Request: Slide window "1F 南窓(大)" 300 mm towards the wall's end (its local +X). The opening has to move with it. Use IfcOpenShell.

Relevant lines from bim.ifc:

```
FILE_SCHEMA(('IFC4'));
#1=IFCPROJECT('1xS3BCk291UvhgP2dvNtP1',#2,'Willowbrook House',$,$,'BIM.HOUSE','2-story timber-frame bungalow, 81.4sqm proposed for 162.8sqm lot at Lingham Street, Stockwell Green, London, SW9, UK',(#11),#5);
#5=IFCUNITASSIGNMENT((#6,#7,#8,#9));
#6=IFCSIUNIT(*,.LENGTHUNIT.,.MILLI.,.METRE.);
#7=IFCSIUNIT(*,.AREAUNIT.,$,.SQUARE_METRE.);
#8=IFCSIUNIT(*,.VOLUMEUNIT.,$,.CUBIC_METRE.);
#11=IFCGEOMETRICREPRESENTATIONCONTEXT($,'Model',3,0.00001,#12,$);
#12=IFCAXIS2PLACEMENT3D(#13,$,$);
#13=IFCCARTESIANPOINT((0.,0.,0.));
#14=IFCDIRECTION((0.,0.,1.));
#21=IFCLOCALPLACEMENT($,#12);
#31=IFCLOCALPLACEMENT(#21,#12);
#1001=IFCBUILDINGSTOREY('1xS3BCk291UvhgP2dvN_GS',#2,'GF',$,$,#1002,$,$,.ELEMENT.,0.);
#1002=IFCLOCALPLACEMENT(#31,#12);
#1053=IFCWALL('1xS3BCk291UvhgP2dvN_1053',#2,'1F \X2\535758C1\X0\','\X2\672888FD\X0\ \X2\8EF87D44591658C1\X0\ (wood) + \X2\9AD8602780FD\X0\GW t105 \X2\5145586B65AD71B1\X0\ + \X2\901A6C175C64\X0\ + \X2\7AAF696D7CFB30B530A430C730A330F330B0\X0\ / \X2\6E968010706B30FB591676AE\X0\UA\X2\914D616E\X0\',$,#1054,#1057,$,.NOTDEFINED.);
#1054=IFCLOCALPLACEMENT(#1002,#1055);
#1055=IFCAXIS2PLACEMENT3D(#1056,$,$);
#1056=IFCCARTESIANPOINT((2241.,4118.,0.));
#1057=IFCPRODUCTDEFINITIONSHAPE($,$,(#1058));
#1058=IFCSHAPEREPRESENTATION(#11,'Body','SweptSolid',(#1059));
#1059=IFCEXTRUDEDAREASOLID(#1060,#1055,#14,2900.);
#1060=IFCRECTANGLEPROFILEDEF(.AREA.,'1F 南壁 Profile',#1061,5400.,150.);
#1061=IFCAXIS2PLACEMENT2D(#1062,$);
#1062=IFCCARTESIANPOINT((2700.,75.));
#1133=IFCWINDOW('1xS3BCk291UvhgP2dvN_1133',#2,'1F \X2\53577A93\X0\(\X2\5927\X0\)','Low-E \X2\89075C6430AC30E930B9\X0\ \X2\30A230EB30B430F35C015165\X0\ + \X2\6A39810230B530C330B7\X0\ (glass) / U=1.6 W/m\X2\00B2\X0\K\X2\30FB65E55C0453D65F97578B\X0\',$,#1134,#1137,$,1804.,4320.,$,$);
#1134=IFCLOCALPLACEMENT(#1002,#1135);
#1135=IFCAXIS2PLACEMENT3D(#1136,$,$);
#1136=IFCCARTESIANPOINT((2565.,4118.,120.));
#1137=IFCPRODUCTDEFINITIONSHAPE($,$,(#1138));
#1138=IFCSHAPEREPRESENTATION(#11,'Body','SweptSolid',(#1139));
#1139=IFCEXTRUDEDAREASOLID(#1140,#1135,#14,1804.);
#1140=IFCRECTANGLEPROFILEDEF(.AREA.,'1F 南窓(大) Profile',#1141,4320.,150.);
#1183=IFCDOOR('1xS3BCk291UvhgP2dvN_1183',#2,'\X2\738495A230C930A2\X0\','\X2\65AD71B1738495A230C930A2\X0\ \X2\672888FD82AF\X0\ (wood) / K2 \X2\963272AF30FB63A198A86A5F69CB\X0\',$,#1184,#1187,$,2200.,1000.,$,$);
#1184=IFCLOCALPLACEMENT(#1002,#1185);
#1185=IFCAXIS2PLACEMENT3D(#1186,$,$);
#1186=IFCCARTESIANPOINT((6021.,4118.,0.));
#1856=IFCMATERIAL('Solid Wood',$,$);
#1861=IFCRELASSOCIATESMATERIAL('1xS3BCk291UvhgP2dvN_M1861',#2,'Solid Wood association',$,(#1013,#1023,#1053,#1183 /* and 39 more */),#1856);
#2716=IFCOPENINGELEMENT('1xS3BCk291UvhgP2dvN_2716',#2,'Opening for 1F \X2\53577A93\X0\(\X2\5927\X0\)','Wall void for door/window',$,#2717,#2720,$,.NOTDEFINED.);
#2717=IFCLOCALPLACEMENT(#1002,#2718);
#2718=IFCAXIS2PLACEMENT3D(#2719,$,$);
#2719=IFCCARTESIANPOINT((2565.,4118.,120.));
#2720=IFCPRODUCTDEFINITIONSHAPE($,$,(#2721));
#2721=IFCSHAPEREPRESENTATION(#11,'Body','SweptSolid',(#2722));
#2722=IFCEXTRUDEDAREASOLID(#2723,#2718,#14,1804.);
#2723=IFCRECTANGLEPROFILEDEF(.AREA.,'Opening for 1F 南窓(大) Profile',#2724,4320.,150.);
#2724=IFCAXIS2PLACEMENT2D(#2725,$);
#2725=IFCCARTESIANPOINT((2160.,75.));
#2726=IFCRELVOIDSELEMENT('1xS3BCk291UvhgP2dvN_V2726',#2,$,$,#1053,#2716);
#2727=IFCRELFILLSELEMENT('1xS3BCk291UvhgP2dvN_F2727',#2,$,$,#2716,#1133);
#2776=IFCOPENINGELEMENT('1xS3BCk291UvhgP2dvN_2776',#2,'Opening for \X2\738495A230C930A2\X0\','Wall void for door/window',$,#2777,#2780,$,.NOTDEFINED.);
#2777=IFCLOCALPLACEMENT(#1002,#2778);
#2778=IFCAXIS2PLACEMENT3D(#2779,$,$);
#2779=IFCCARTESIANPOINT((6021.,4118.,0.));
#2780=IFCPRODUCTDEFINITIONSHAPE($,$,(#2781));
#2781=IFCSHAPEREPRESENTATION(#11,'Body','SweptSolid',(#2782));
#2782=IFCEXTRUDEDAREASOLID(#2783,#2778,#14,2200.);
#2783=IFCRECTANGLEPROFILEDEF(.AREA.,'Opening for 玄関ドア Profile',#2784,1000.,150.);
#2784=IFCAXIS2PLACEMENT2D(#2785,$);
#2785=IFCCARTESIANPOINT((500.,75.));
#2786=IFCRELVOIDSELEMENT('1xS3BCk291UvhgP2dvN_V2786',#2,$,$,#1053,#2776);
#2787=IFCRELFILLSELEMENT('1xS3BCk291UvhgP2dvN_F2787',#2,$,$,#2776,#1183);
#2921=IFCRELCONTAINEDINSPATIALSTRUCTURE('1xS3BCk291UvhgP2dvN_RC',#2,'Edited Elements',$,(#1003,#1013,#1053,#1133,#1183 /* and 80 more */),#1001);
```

```python
import ifcopenshell
import ifcopenshell.api.geometry
import ifcopenshell.util.placement
import ifcopenshell.util.unit

model = ifcopenshell.open("bim.ifc")
unit_scale = ifcopenshell.util.unit.calculate_unit_scale(model)

window = model.by_id(1133)
opening = window.FillsVoids[0].RelatingOpeningElement
wall = opening.VoidsElements[0].RelatingBuildingElement

wall_matrix = ifcopenshell.util.placement.get_local_placement(wall.ObjectPlacement)
shift = wall_matrix[:3, 0] * 0.3 / unit_scale
before = ifcopenshell.util.placement.get_local_placement(window.ObjectPlacement)[:3, 3].copy()

# The window is not placed relative to its opening, so move both.
for product in (opening, window):
    matrix = ifcopenshell.util.placement.get_local_placement(product.ObjectPlacement)
    matrix[:3, 3] += shift
    ifcopenshell.api.geometry.edit_object_placement(model, product=product, matrix=matrix, is_si=False)

after = ifcopenshell.util.placement.get_local_placement(window.ObjectPlacement)[:3, 3]
print("window moved by", (after - before).round(3) + 0.0)

model.write("bim-out.ifc")
```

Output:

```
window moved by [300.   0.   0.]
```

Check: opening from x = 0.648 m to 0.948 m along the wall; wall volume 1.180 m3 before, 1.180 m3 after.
